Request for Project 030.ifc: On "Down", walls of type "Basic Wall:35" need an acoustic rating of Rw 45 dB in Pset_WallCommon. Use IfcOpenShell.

First a look at what the model holds.

```python
import ifcopenshell
import ifcopenshell.util.element

model = ifcopenshell.open("Project 030.ifc")
print(model.schema)
storey = next(s for s in model.by_type("IfcBuildingStorey") if s.Name == "Down")
walls = [e for e in ifcopenshell.util.element.get_decomposition(storey) if e.is_a("IfcWall")]
seen = {}
for e in walls:
    element_type = ifcopenshell.util.element.get_type(e)
    key = (element_type.Name if element_type != e and element_type else None, ifcopenshell.util.element.get_pset(e, "Pset_WallCommon", "AcousticRating"))
    seen[key] = seen.get(key, 0) + 1
for (name, value), count in sorted(seen.items(), key=str):
    print(count, "x", name, "|", value)
```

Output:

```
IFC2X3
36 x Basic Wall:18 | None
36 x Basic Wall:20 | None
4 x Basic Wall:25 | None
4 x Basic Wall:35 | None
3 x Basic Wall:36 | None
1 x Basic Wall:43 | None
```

```python
import ifcopenshell
import ifcopenshell.api.pset
import ifcopenshell.util.element

model = ifcopenshell.open("Project 030.ifc")

storey = next(s for s in model.by_type("IfcBuildingStorey") if s.Name == "Down")
walls = [e for e in ifcopenshell.util.element.get_decomposition(storey) if e.is_a("IfcWall")]

count = 0
for e in walls:
    element_type = ifcopenshell.util.element.get_type(e)
    if element_type in (None, e) or element_type.Name != "Basic Wall:35":
        continue
    # add_pset returns the element's existing set when there is one.
    pset = ifcopenshell.api.pset.add_pset(model, product=e, name="Pset_WallCommon")
    ifcopenshell.api.pset.edit_pset(model, pset=pset, properties={"AcousticRating": "Rw 45 dB"})
    count += 1

print(count, "walls updated")

model.write("Project 030_rev.ifc")
```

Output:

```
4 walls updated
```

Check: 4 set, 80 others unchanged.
